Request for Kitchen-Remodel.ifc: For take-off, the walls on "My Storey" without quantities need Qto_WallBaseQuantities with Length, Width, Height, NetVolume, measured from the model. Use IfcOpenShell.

First a look at what the model holds.

```python
import ifcopenshell
import ifcopenshell.util.element
import ifcopenshell.util.unit

model = ifcopenshell.open("Kitchen-Remodel.ifc")
print(model.schema)
for unit_type in ("LENGTHUNIT", "AREAUNIT", "VOLUMEUNIT"):
    print(unit_type, ifcopenshell.util.unit.calculate_unit_scale(model, unit_type))
storey = next(s for s in model.by_type("IfcBuildingStorey") if s.Name == "My Storey")
walls = [e for e in ifcopenshell.util.element.get_decomposition(storey) if e.is_a("IfcWall")]
for e in sorted(walls, key=lambda e: e.id()):
    print(e.id(), e.is_a(), e.Name, list(ifcopenshell.util.element.get_psets(e, qtos_only=True)), sep=" | ")
```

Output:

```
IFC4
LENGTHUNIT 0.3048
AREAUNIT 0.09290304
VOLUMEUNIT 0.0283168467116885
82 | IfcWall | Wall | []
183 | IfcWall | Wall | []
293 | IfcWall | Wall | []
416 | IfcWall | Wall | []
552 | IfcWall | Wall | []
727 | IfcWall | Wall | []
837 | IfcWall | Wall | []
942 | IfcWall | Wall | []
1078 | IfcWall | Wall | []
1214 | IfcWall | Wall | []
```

```python
import ifcopenshell
import ifcopenshell.api.pset
import ifcopenshell.geom
import ifcopenshell.util.element
import ifcopenshell.util.shape
import ifcopenshell.util.unit

model = ifcopenshell.open("Kitchen-Remodel.ifc")
unit_scale = ifcopenshell.util.unit.calculate_unit_scale(model)
volume_scale = ifcopenshell.util.unit.calculate_unit_scale(model, "VOLUMEUNIT")
settings = ifcopenshell.geom.settings()

storey = next(s for s in model.by_type("IfcBuildingStorey") if s.Name == "My Storey")
walls = [e for e in ifcopenshell.util.element.get_decomposition(storey) if e.is_a("IfcWall")]

for e in sorted(walls, key=lambda e: e.id()):
    if ifcopenshell.util.element.get_psets(e, qtos_only=True, should_inherit=False):
        continue
    # Geometry comes back in metres, in the element's own axes.
    shape = ifcopenshell.geom.create_shape(settings, e)
    values = {
        "Length": ifcopenshell.util.shape.get_x(shape.geometry) / unit_scale,
        "Width": ifcopenshell.util.shape.get_y(shape.geometry) / unit_scale,
        "Height": ifcopenshell.util.shape.get_z(shape.geometry) / unit_scale,
        "NetVolume": ifcopenshell.util.shape.get_volume(shape.geometry) / volume_scale,
    }
    qto = ifcopenshell.api.pset.add_qto(model, product=e, name="Qto_WallBaseQuantities")
    ifcopenshell.api.pset.edit_qto(model, qto=qto, properties=values)
    print(e.id(), {k: round(v, 3) for k, v in values.items()})

model.write("Kitchen-Remodel_edited.ifc")
```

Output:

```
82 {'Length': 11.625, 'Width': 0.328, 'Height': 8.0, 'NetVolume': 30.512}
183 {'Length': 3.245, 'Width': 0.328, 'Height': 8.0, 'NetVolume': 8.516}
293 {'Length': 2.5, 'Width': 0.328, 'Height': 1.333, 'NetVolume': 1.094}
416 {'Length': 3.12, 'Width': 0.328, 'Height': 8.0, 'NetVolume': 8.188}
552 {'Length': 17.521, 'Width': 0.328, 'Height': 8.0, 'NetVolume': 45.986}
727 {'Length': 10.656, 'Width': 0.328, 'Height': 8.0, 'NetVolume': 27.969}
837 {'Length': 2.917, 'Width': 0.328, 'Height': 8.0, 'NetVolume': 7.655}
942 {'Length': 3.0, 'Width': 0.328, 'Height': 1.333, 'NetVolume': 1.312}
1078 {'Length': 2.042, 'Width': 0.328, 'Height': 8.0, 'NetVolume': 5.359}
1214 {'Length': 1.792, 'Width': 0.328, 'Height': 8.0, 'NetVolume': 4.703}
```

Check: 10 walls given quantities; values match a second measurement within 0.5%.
